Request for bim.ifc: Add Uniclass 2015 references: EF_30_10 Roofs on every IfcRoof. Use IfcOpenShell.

First a look at what the model holds.

```python
import ifcopenshell

model = ifcopenshell.open("bim.ifc")
print(model.schema)
print("classifications:", [c.Name for c in model.by_type("IfcClassification")])
for ifc_class in ("IfcDoor", "IfcRoof", "IfcStair", "IfcWall", "IfcWindow"):
    print(ifc_class, len(model.by_type(ifc_class)))
```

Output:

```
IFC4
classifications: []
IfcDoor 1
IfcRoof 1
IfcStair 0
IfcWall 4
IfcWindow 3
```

```python
import ifcopenshell
import ifcopenshell.api.classification

model = ifcopenshell.open("bim.ifc")

system = ifcopenshell.api.classification.add_classification(model, classification="Uniclass 2015")

codes = {
    "IfcRoof": ("EF_30_10", "Roofs"),
}
for ifc_class, (code, name) in codes.items():
    products = model.by_type(ifc_class)
    ifcopenshell.api.classification.add_reference(
        model, products=products, classification=system, identification=code, name=name
    )
    print(code, len(products))

model.write("bim-out.ifc")
```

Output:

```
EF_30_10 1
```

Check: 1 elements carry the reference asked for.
